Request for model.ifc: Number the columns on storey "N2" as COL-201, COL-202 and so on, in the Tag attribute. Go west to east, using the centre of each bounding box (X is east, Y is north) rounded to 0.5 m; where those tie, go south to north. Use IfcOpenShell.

First a look at what the model holds.

```python
import ifcopenshell
import ifcopenshell.util.element
import ifcopenshell.util.placement

model = ifcopenshell.open("model.ifc")
print(model.schema)
storey = next(s for s in model.by_type("IfcBuildingStorey") if s.Name == "N2")
columns = [e for e in ifcopenshell.util.element.get_decomposition(storey) if e.is_a("IfcColumn")]
for e in sorted(columns, key=lambda e: e.id()):
    origin = ifcopenshell.util.placement.get_local_placement(e.ObjectPlacement)[:3, 3]
    print(e.id(), e.Tag, e.Name, origin.round(2) + 0.0, sep=" | ")
```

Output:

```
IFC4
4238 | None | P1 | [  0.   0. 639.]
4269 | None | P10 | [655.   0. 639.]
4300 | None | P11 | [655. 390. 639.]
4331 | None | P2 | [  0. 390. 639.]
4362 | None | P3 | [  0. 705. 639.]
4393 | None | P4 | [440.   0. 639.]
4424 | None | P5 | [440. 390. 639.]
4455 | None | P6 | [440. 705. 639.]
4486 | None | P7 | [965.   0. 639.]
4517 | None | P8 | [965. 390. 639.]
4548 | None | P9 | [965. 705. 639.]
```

```python
import ifcopenshell
import ifcopenshell.geom
import ifcopenshell.util.element
import ifcopenshell.util.shape

model = ifcopenshell.open("model.ifc")
settings = ifcopenshell.geom.settings()
settings.set("use-world-coords", True)


def centre(element):
    shape = ifcopenshell.geom.create_shape(settings, element)
    return ifcopenshell.util.shape.get_bbox_centroid(shape.geometry)


storey = next(s for s in model.by_type("IfcBuildingStorey") if s.Name == "N2")
columns = [e for e in ifcopenshell.util.element.get_decomposition(storey) if e.is_a("IfcColumn")]

# Insertion points can sit at a corner or the storey origin, so sort by the geometry (in metres).
centres = {e: centre(e) for e in columns}
columns.sort(key=lambda e: (round(centres[e][0] / 0.5), centres[e][1]))

for i, e in enumerate(columns, start=1):
    number = f"COL-2{i:02d}"
    e.Tag = number
    print(e.id(), number)

model.write("model_v2.ifc")
```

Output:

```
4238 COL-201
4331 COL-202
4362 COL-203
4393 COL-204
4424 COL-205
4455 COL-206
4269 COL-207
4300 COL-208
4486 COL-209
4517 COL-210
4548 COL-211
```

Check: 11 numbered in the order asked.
